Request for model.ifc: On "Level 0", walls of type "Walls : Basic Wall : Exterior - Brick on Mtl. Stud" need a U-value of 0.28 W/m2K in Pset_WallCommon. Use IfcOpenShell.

First a look at what the model holds.

```python
import ifcopenshell
import ifcopenshell.util.element

model = ifcopenshell.open("model.ifc")
print(model.schema)
storey = next(s for s in model.by_type("IfcBuildingStorey") if s.Name == "Level 0")
walls = [e for e in ifcopenshell.util.element.get_decomposition(storey) if e.is_a("IfcWall")]
seen = {}
for e in walls:
    element_type = ifcopenshell.util.element.get_type(e)
    key = (element_type.Name if element_type != e and element_type else None, ifcopenshell.util.element.get_pset(e, "Pset_WallCommon", "ThermalTransmittance"))
    seen[key] = seen.get(key, 0) + 1
for (name, value), count in sorted(seen.items(), key=str):
    print(count, "x", name, "|", value)
```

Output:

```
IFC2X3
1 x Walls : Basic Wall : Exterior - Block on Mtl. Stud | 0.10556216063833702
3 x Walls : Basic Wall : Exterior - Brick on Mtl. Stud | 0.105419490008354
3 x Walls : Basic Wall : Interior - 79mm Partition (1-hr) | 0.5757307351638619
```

```python
import ifcopenshell
import ifcopenshell.api.pset
import ifcopenshell.util.element

model = ifcopenshell.open("model.ifc")

storey = next(s for s in model.by_type("IfcBuildingStorey") if s.Name == "Level 0")
walls = [e for e in ifcopenshell.util.element.get_decomposition(storey) if e.is_a("IfcWall")]

count = 0
for e in walls:
    element_type = ifcopenshell.util.element.get_type(e)
    if element_type in (None, e) or element_type.Name != "Walls : Basic Wall : Exterior - Brick on Mtl. Stud":
        continue
    # add_pset returns the element's existing set when there is one.
    pset = ifcopenshell.api.pset.add_pset(model, product=e, name="Pset_WallCommon")
    ifcopenshell.api.pset.edit_pset(model, pset=pset, properties={"ThermalTransmittance": 0.28})
    count += 1

print(count, "walls updated")

model.write("model_rev.ifc")
```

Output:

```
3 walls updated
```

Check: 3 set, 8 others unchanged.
